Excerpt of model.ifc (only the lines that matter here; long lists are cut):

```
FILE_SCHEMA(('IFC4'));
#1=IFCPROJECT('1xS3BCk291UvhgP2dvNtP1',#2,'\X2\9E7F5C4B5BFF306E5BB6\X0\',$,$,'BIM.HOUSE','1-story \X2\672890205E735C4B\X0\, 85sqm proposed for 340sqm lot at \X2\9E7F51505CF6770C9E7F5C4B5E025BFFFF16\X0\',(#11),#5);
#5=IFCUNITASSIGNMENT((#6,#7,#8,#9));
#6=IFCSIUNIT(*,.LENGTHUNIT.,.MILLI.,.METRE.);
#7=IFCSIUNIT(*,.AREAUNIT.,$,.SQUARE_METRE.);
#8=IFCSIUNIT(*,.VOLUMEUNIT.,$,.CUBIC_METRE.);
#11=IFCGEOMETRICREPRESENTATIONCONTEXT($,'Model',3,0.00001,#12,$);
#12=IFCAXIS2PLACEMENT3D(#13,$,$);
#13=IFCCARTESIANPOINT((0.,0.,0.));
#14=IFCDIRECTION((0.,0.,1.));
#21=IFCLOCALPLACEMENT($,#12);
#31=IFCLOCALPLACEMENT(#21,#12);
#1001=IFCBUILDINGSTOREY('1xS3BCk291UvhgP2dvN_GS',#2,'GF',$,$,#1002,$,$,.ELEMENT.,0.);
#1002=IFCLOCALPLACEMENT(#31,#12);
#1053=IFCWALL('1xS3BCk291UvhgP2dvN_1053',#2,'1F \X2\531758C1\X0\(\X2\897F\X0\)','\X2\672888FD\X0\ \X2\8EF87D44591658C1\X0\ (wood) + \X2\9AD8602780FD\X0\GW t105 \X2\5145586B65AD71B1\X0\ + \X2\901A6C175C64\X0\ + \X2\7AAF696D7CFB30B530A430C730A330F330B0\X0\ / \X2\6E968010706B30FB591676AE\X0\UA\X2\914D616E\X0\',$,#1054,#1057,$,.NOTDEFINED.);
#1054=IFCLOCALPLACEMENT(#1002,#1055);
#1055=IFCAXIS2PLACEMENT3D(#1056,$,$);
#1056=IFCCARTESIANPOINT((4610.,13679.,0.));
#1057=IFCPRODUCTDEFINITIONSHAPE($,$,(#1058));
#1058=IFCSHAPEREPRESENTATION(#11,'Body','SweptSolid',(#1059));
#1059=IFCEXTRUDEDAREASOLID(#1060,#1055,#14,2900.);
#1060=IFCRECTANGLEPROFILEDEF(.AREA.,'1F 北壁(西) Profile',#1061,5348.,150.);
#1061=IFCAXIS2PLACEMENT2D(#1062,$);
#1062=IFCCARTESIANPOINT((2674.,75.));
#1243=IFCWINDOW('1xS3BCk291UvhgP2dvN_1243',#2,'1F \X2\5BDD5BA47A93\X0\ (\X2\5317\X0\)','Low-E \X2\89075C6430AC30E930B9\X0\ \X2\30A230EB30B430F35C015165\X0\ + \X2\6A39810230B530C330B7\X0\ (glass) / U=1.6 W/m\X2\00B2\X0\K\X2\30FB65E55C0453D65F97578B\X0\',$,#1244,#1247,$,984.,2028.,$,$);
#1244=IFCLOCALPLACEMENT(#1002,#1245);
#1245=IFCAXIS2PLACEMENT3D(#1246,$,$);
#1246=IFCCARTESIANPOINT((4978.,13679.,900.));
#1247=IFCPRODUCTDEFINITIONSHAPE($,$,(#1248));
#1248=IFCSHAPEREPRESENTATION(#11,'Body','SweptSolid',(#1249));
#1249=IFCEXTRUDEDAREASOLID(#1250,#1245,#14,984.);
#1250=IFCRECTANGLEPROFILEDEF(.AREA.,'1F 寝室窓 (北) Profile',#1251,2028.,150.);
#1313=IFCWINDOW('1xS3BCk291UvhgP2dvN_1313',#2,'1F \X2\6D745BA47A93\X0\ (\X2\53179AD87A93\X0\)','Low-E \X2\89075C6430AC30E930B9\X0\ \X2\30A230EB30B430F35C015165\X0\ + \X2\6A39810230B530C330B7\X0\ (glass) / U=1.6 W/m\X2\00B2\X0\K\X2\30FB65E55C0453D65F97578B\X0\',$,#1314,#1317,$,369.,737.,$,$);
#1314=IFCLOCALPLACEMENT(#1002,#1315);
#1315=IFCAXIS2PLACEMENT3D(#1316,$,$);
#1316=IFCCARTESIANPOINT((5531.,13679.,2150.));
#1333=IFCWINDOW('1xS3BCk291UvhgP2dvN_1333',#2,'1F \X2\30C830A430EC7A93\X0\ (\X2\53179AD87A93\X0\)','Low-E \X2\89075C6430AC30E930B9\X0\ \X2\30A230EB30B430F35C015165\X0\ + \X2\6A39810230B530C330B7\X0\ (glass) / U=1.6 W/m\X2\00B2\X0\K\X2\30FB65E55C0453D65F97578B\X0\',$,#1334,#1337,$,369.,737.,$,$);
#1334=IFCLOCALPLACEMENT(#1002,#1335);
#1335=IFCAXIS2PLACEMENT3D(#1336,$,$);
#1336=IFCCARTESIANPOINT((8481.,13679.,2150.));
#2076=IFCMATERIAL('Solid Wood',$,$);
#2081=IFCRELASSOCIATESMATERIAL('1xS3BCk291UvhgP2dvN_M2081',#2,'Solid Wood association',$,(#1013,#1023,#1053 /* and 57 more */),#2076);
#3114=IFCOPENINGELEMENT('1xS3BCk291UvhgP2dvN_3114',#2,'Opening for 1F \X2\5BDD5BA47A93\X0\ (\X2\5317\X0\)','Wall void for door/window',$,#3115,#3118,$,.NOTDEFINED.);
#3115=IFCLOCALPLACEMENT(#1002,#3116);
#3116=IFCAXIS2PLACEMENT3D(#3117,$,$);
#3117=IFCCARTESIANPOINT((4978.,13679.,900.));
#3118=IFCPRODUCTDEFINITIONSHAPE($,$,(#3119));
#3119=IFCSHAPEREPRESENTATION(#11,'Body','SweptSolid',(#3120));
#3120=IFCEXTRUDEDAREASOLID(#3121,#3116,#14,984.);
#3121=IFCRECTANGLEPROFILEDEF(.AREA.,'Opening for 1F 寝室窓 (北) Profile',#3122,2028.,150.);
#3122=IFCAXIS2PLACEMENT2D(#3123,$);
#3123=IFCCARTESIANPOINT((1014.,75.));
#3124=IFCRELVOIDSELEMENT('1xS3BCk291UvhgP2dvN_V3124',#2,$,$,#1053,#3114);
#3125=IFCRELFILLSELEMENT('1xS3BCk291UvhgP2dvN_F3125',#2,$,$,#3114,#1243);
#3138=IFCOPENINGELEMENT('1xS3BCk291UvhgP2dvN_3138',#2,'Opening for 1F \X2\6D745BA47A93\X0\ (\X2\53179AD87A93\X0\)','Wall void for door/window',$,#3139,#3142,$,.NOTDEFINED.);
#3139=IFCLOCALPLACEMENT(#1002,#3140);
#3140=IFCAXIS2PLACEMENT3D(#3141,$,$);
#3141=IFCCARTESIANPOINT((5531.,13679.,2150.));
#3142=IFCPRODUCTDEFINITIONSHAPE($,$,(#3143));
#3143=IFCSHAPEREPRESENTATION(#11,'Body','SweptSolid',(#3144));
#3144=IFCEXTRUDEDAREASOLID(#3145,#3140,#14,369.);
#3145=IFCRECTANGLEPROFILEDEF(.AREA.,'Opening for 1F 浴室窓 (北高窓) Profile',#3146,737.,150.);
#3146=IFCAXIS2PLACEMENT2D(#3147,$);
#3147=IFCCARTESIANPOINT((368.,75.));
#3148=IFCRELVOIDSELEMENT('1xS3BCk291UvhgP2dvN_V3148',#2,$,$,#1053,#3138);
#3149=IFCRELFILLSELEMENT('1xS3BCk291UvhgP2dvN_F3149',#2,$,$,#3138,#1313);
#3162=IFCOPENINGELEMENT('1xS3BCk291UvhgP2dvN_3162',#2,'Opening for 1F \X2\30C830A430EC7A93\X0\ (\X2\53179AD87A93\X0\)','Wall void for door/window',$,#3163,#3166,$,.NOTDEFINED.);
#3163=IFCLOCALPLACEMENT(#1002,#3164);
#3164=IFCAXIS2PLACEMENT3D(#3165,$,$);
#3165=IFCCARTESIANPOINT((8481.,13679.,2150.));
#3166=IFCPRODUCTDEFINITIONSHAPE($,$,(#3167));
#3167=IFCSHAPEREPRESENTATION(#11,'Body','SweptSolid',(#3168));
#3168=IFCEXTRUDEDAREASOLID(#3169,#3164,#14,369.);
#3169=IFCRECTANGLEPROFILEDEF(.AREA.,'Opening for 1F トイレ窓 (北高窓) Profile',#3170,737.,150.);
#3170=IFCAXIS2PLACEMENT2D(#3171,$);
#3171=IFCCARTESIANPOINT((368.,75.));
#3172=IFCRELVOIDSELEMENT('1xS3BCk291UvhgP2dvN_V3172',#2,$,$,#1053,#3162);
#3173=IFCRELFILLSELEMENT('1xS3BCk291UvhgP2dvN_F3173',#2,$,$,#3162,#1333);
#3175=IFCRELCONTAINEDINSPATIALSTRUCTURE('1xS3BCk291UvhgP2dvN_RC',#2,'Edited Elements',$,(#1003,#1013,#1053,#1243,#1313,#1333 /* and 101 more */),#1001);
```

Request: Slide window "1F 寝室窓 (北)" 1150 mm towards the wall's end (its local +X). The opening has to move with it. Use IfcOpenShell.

```python
import ifcopenshell
import ifcopenshell.api.geometry
import ifcopenshell.util.placement
import ifcopenshell.util.unit

model = ifcopenshell.open("model.ifc")
unit_scale = ifcopenshell.util.unit.calculate_unit_scale(model)

window = model.by_guid("1xS3BCk291UvhgP2dvN_1243")
opening = window.FillsVoids[0].RelatingOpeningElement
wall = opening.VoidsElements[0].RelatingBuildingElement

wall_matrix = ifcopenshell.util.placement.get_local_placement(wall.ObjectPlacement)
shift = wall_matrix[:3, 0] * 1.15 / unit_scale
before = ifcopenshell.util.placement.get_local_placement(window.ObjectPlacement)[:3, 3].copy()

# The window is not placed relative to its opening, so move both.
for product in (opening, window):
    matrix = ifcopenshell.util.placement.get_local_placement(product.ObjectPlacement)
    matrix[:3, 3] += shift
    ifcopenshell.api.geometry.edit_object_placement(model, product=product, matrix=matrix, is_si=False)

after = ifcopenshell.util.placement.get_local_placement(window.ObjectPlacement)[:3, 3]
print("window moved by", (after - before).round(3) + 0.0)

model.write("model_edited.ifc")
```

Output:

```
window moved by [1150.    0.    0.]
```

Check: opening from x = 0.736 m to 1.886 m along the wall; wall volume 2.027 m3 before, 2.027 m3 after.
